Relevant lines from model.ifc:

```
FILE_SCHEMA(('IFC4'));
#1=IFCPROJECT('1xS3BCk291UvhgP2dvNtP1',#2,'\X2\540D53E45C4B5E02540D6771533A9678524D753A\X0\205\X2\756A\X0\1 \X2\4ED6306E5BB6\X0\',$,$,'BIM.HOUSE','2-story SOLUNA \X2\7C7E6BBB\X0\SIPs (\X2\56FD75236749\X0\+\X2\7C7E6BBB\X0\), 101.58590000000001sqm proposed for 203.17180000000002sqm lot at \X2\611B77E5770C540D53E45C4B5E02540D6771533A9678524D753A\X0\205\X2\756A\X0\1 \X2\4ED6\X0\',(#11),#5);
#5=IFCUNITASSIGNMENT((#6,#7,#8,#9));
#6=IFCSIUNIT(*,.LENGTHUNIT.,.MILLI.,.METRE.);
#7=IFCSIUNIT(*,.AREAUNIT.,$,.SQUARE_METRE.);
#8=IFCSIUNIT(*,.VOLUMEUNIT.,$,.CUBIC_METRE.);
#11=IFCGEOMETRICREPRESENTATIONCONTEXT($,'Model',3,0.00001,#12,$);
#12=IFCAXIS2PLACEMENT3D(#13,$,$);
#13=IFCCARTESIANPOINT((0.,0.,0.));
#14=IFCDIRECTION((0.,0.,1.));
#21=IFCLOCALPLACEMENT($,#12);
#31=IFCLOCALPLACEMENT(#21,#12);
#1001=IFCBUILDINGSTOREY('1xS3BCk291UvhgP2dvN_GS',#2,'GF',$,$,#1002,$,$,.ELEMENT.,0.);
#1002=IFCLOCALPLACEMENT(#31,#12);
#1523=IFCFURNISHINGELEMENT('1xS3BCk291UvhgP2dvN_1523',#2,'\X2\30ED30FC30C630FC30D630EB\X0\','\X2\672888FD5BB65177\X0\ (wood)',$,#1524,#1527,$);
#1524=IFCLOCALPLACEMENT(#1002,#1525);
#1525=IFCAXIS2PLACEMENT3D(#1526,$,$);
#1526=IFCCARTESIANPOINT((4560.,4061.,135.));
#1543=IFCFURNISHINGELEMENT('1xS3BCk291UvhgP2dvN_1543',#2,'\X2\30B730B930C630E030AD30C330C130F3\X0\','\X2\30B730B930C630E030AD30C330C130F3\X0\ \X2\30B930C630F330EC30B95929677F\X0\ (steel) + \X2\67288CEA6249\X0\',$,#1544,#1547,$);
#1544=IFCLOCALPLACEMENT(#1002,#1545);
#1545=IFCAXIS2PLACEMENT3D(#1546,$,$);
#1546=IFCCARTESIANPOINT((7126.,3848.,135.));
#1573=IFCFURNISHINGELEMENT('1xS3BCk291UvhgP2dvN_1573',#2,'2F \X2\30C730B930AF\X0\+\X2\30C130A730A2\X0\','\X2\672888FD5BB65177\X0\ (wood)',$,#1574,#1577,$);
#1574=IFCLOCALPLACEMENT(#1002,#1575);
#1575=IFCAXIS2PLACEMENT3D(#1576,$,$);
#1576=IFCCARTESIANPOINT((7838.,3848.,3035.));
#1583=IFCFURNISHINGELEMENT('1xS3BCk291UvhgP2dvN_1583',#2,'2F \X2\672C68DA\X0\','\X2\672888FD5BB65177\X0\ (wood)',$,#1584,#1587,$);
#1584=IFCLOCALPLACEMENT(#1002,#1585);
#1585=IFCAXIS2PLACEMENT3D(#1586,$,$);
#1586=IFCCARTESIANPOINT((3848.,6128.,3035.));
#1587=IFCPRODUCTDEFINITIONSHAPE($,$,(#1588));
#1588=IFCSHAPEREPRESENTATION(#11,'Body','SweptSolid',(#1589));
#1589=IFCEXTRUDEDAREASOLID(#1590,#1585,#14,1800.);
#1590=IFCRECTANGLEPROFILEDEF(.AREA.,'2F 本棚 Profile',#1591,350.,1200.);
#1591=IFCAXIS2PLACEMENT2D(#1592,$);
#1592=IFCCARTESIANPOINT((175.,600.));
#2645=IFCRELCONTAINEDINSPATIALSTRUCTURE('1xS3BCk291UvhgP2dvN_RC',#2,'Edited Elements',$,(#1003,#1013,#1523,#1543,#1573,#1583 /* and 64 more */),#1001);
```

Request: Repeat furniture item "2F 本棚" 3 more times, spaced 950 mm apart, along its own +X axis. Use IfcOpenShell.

```python
import ifcopenshell
import ifcopenshell.api.geometry
import ifcopenshell.api.root
import ifcopenshell.util.element
import ifcopenshell.util.placement
import ifcopenshell.util.unit

model = ifcopenshell.open("model.ifc")
unit_scale = ifcopenshell.util.unit.calculate_unit_scale(model)


def reuse_history(source, copy):
    """copy_class also copies each property set's owner history, people and application; keep the originals."""
    for rel in copy.IsDefinedBy:
        if rel.is_a("IfcRelDefinesByProperties") and (history := rel.RelatingPropertyDefinition.OwnerHistory):
            rel.RelatingPropertyDefinition.OwnerHistory = source.OwnerHistory
            ifcopenshell.util.element.remove_deep2(model, history)


source = model.by_guid("1xS3BCk291UvhgP2dvN_1583")
base = ifcopenshell.util.placement.get_local_placement(source.ObjectPlacement)
step = base[:3, 0] * 0.95 / unit_scale

for i in range(1, 4):
    copy = ifcopenshell.api.root.copy_class(model, product=source)
    copy.Representation = ifcopenshell.util.element.copy_deep(
        model, source.Representation, exclude=["IfcGeometricRepresentationContext", "IfcRepresentationMap"]
    )
    reuse_history(source, copy)
    matrix = base.copy()
    matrix[:3, 3] += i * step
    print("added at", matrix[:3, 3].round(3) + 0.0)
    ifcopenshell.api.geometry.edit_object_placement(model, product=copy, matrix=matrix, is_si=False)

model.write("model_updated.ifc")
```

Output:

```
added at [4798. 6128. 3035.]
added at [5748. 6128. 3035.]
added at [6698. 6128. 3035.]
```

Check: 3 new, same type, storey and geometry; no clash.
